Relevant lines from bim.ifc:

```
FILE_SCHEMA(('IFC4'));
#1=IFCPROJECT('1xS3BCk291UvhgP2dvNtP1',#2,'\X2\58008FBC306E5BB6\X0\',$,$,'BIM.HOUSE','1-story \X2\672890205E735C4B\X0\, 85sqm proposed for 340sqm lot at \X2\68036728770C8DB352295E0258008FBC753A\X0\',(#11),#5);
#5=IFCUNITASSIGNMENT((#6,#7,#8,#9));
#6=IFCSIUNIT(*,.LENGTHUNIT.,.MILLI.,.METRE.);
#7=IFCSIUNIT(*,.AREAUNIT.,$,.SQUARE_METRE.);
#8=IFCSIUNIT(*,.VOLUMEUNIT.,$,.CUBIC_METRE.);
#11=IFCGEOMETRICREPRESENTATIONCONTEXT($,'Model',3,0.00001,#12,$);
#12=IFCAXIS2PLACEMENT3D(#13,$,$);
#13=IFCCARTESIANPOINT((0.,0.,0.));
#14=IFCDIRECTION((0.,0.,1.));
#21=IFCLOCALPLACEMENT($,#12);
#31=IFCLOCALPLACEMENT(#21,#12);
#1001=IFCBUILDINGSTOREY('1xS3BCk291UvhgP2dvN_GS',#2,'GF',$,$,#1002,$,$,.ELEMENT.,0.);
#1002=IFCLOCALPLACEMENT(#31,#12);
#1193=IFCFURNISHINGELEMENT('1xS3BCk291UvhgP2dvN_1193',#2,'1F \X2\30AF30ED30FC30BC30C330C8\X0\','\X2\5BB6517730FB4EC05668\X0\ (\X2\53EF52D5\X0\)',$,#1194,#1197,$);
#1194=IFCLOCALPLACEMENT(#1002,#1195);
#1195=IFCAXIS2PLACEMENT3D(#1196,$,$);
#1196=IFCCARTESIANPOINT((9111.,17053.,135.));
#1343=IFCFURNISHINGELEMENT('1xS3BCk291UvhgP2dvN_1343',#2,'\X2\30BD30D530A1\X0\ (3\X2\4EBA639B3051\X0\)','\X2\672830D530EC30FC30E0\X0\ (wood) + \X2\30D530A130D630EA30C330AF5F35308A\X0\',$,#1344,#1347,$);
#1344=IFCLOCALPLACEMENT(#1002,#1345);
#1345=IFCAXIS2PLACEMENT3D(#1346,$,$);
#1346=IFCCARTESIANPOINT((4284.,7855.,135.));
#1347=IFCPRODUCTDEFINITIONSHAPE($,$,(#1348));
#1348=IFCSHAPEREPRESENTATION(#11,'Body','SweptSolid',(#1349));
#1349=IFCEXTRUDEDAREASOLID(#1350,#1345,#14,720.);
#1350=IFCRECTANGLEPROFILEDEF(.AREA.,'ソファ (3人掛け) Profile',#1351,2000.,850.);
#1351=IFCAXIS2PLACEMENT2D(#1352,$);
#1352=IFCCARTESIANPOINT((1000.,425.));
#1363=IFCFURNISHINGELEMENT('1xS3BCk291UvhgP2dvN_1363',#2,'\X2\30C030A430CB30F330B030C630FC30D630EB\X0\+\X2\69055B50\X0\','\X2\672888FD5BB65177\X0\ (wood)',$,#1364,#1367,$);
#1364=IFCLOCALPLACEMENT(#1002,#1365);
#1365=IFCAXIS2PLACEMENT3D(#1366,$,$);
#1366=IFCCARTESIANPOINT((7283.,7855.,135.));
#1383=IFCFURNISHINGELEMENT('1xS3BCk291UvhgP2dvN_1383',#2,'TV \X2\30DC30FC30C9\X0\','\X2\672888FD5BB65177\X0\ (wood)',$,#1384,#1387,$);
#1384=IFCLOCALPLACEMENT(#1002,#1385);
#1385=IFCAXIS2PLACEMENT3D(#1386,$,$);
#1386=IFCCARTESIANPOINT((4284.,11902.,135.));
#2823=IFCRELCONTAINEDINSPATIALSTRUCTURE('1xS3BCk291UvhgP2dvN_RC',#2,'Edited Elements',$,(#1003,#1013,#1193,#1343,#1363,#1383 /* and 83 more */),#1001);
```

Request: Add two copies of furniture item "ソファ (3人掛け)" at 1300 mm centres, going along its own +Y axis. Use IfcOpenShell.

```python
import ifcopenshell
import ifcopenshell.api.geometry
import ifcopenshell.api.root
import ifcopenshell.util.element
import ifcopenshell.util.placement

model = ifcopenshell.open("bim.ifc")


def reuse_history(source, copy):
    """copy_class also copies each property set's owner history, people and application; keep the originals."""
    for rel in copy.IsDefinedBy:
        if rel.is_a("IfcRelDefinesByProperties") and (history := rel.RelatingPropertyDefinition.OwnerHistory):
            rel.RelatingPropertyDefinition.OwnerHistory = source.OwnerHistory
            ifcopenshell.util.element.remove_deep2(model, history)


source = model.by_id(1343)
base = ifcopenshell.util.placement.get_local_placement(source.ObjectPlacement)
step = base[:3, 1] * 1300.0

for i in range(1, 3):
    copy = ifcopenshell.api.root.copy_class(model, product=source)
    copy.Representation = ifcopenshell.util.element.copy_deep(
        model, source.Representation, exclude=["IfcGeometricRepresentationContext", "IfcRepresentationMap"]
    )
    reuse_history(source, copy)
    matrix = base.copy()
    matrix[:3, 3] += i * step
    print("added at", matrix[:3, 3].round(3) + 0.0)
    ifcopenshell.api.geometry.edit_object_placement(model, product=copy, matrix=matrix, is_si=False)

model.write("bim_edited.ifc")
```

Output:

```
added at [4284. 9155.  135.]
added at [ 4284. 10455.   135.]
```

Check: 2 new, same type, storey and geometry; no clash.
